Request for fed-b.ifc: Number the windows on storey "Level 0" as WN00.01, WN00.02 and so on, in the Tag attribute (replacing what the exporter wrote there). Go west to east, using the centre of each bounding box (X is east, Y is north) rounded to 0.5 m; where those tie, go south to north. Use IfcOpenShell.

First a look at what the model holds.

```python
import ifcopenshell
import ifcopenshell.util.element
import ifcopenshell.util.placement

model = ifcopenshell.open("fed-b.ifc")
print(model.schema)
storey = next(s for s in model.by_type("IfcBuildingStorey") if s.Name == "Level 0")
windows = [e for e in ifcopenshell.util.element.get_decomposition(storey) if e.is_a("IfcWindow")]
for e in sorted(windows, key=lambda e: e.id()):
    origin = ifcopenshell.util.placement.get_local_placement(e.ObjectPlacement)[:3, 3]
    print(e.id(), e.Tag, e.Name, origin.round(2) + 0.0, sep=" | ")
```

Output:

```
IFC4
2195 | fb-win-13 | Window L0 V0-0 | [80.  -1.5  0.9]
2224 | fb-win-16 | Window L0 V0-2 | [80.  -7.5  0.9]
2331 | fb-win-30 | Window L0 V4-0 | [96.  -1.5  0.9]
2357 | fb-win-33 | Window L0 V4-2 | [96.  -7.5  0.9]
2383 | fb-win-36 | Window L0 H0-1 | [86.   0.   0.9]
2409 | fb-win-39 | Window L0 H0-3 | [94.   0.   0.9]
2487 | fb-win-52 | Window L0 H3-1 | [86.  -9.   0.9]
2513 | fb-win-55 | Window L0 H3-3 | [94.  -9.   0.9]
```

```python
import ifcopenshell
import ifcopenshell.geom
import ifcopenshell.util.element
import ifcopenshell.util.shape

model = ifcopenshell.open("fed-b.ifc")
settings = ifcopenshell.geom.settings()
settings.set("use-world-coords", True)


def centre(element):
    shape = ifcopenshell.geom.create_shape(settings, element)
    return ifcopenshell.util.shape.get_bbox_centroid(shape.geometry)


storey = next(s for s in model.by_type("IfcBuildingStorey") if s.Name == "Level 0")
windows = [e for e in ifcopenshell.util.element.get_decomposition(storey) if e.is_a("IfcWindow")]

# Insertion points can sit at a corner or the storey origin, so sort by the geometry (in metres).
centres = {e: centre(e) for e in windows}
windows.sort(key=lambda e: (round(centres[e][0] / 0.5), centres[e][1]))

for i, e in enumerate(windows, start=1):
    number = f"WN00.{i:02d}"
    e.Tag = number
    print(e.id(), number)

model.write("fed-b_v2.ifc")
```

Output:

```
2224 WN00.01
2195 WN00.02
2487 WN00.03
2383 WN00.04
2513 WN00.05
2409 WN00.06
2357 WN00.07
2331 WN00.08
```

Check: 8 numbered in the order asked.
